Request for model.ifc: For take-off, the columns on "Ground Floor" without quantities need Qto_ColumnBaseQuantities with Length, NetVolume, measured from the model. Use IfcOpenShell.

First a look at what the model holds.

```python
import ifcopenshell
import ifcopenshell.util.element
import ifcopenshell.util.unit

model = ifcopenshell.open("model.ifc")
print(model.schema)
for unit_type in ("LENGTHUNIT", "AREAUNIT", "VOLUMEUNIT"):
    print(unit_type, ifcopenshell.util.unit.calculate_unit_scale(model, unit_type))
storey = next(s for s in model.by_type("IfcBuildingStorey") if s.Name == "Ground Floor")
columns = [e for e in ifcopenshell.util.element.get_decomposition(storey) if e.is_a("IfcColumn")]
for e in sorted(columns, key=lambda e: e.id()):
    print(e.id(), e.is_a(), e.Name, list(ifcopenshell.util.element.get_psets(e, qtos_only=True)), sep=" | ")
```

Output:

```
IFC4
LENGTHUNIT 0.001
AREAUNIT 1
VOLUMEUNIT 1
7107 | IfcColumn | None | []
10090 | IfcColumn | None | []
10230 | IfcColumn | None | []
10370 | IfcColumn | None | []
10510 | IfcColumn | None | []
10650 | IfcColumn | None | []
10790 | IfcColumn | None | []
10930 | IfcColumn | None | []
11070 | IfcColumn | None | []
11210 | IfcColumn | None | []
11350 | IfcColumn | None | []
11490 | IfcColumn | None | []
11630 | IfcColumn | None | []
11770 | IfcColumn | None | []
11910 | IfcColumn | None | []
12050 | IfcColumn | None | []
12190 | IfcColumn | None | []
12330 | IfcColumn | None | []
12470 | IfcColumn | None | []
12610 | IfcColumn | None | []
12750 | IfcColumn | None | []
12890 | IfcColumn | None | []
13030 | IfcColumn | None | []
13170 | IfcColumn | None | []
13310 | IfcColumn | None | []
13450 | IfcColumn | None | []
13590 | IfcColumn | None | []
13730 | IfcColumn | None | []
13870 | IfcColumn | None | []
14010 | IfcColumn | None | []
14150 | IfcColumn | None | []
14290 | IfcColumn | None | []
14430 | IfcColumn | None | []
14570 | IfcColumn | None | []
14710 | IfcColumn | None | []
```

```python
import ifcopenshell
import ifcopenshell.api.pset
import ifcopenshell.geom
import ifcopenshell.util.element
import ifcopenshell.util.shape
import ifcopenshell.util.unit

model = ifcopenshell.open("model.ifc")
unit_scale = ifcopenshell.util.unit.calculate_unit_scale(model)
volume_scale = ifcopenshell.util.unit.calculate_unit_scale(model, "VOLUMEUNIT")
settings = ifcopenshell.geom.settings()

storey = next(s for s in model.by_type("IfcBuildingStorey") if s.Name == "Ground Floor")
columns = [e for e in ifcopenshell.util.element.get_decomposition(storey) if e.is_a("IfcColumn")]

for e in sorted(columns, key=lambda e: e.id()):
    if ifcopenshell.util.element.get_psets(e, qtos_only=True, should_inherit=False):
        continue
    # Geometry comes back in metres, in the element's own axes.
    shape = ifcopenshell.geom.create_shape(settings, e)
    values = {
        "Length": ifcopenshell.util.shape.get_z(shape.geometry) / unit_scale,
        "NetVolume": ifcopenshell.util.shape.get_volume(shape.geometry) / volume_scale,
    }
    qto = ifcopenshell.api.pset.add_qto(model, product=e, name="Qto_ColumnBaseQuantities")
    ifcopenshell.api.pset.edit_qto(model, qto=qto, properties=values)
    print(e.id(), {k: round(v, 3) for k, v in values.items()})

model.write("model_rev.ifc")
```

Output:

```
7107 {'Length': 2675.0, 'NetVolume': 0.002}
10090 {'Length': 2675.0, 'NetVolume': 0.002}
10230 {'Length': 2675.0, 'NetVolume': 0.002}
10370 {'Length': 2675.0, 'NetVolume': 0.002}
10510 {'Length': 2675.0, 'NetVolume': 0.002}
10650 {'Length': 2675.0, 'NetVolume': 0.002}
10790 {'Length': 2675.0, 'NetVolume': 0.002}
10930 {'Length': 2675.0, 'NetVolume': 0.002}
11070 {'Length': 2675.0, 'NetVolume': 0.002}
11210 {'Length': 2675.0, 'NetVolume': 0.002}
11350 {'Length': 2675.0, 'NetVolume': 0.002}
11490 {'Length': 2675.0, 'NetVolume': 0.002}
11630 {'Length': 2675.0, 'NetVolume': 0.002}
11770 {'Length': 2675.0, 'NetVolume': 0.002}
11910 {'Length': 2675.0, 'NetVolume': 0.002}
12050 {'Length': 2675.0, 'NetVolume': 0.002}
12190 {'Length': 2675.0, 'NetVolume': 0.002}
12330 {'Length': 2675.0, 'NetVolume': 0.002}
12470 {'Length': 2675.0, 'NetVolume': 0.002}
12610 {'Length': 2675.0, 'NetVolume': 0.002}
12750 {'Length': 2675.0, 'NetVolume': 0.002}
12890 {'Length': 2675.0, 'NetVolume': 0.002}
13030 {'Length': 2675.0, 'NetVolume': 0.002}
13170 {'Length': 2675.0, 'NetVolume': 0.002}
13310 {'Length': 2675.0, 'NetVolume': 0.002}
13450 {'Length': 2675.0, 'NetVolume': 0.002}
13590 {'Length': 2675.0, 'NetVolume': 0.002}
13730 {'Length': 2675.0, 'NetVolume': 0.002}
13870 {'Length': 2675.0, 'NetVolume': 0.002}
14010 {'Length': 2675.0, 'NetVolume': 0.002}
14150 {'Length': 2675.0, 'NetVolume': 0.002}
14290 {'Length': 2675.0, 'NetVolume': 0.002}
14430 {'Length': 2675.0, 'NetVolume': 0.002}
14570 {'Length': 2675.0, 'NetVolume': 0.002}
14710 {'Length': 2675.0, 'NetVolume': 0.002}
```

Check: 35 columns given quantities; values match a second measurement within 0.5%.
